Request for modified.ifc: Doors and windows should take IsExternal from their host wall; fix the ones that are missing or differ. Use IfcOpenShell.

First a look at what the model holds.

```python
import ifcopenshell
import ifcopenshell.util.element

model = ifcopenshell.open("modified.ifc")
print(model.schema)
seen = {}
for e in model.by_type("IfcDoor") + model.by_type("IfcWindow"):
    if not e.FillsVoids:
        continue
    host = e.FillsVoids[0].RelatingOpeningElement.VoidsElements[0].RelatingBuildingElement
    own = ifcopenshell.util.element.get_pset(e, f"Pset_{e.is_a()[3:].removesuffix('StandardCase')}Common", "IsExternal")
    wall = ifcopenshell.util.element.get_pset(host, "Pset_WallCommon", "IsExternal")
    seen[e.is_a(), own, wall] = seen.get((e.is_a(), own, wall), 0) + 1
for (cls, own, wall), count in sorted(seen.items(), key=str):
    print(count, cls, "IsExternal:", own, "| host wall:", wall)
```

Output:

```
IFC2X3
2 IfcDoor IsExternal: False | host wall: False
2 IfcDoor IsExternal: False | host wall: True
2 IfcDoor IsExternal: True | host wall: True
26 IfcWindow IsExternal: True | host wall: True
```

```python
import ifcopenshell
import ifcopenshell.api.pset
import ifcopenshell.util.element

model = ifcopenshell.open("modified.ifc")

count = 0
for ifc_class, pset_name in (("IfcDoor", "Pset_DoorCommon"), ("IfcWindow", "Pset_WindowCommon")):
    for e in model.by_type(ifc_class):
        if not e.FillsVoids:
            continue
        host = e.FillsVoids[0].RelatingOpeningElement.VoidsElements[0].RelatingBuildingElement
        external = ifcopenshell.util.element.get_pset(host, "Pset_WallCommon", "IsExternal")
        if external is None or ifcopenshell.util.element.get_pset(e, pset_name, "IsExternal") == external:
            continue
        pset = ifcopenshell.api.pset.add_pset(model, product=e, name=pset_name)
        ifcopenshell.api.pset.edit_pset(model, pset=pset, properties={"IsExternal": external})
        count += 1

print(count, "updated")

model.write("modified_rev.ifc")
```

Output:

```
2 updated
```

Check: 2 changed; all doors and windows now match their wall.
